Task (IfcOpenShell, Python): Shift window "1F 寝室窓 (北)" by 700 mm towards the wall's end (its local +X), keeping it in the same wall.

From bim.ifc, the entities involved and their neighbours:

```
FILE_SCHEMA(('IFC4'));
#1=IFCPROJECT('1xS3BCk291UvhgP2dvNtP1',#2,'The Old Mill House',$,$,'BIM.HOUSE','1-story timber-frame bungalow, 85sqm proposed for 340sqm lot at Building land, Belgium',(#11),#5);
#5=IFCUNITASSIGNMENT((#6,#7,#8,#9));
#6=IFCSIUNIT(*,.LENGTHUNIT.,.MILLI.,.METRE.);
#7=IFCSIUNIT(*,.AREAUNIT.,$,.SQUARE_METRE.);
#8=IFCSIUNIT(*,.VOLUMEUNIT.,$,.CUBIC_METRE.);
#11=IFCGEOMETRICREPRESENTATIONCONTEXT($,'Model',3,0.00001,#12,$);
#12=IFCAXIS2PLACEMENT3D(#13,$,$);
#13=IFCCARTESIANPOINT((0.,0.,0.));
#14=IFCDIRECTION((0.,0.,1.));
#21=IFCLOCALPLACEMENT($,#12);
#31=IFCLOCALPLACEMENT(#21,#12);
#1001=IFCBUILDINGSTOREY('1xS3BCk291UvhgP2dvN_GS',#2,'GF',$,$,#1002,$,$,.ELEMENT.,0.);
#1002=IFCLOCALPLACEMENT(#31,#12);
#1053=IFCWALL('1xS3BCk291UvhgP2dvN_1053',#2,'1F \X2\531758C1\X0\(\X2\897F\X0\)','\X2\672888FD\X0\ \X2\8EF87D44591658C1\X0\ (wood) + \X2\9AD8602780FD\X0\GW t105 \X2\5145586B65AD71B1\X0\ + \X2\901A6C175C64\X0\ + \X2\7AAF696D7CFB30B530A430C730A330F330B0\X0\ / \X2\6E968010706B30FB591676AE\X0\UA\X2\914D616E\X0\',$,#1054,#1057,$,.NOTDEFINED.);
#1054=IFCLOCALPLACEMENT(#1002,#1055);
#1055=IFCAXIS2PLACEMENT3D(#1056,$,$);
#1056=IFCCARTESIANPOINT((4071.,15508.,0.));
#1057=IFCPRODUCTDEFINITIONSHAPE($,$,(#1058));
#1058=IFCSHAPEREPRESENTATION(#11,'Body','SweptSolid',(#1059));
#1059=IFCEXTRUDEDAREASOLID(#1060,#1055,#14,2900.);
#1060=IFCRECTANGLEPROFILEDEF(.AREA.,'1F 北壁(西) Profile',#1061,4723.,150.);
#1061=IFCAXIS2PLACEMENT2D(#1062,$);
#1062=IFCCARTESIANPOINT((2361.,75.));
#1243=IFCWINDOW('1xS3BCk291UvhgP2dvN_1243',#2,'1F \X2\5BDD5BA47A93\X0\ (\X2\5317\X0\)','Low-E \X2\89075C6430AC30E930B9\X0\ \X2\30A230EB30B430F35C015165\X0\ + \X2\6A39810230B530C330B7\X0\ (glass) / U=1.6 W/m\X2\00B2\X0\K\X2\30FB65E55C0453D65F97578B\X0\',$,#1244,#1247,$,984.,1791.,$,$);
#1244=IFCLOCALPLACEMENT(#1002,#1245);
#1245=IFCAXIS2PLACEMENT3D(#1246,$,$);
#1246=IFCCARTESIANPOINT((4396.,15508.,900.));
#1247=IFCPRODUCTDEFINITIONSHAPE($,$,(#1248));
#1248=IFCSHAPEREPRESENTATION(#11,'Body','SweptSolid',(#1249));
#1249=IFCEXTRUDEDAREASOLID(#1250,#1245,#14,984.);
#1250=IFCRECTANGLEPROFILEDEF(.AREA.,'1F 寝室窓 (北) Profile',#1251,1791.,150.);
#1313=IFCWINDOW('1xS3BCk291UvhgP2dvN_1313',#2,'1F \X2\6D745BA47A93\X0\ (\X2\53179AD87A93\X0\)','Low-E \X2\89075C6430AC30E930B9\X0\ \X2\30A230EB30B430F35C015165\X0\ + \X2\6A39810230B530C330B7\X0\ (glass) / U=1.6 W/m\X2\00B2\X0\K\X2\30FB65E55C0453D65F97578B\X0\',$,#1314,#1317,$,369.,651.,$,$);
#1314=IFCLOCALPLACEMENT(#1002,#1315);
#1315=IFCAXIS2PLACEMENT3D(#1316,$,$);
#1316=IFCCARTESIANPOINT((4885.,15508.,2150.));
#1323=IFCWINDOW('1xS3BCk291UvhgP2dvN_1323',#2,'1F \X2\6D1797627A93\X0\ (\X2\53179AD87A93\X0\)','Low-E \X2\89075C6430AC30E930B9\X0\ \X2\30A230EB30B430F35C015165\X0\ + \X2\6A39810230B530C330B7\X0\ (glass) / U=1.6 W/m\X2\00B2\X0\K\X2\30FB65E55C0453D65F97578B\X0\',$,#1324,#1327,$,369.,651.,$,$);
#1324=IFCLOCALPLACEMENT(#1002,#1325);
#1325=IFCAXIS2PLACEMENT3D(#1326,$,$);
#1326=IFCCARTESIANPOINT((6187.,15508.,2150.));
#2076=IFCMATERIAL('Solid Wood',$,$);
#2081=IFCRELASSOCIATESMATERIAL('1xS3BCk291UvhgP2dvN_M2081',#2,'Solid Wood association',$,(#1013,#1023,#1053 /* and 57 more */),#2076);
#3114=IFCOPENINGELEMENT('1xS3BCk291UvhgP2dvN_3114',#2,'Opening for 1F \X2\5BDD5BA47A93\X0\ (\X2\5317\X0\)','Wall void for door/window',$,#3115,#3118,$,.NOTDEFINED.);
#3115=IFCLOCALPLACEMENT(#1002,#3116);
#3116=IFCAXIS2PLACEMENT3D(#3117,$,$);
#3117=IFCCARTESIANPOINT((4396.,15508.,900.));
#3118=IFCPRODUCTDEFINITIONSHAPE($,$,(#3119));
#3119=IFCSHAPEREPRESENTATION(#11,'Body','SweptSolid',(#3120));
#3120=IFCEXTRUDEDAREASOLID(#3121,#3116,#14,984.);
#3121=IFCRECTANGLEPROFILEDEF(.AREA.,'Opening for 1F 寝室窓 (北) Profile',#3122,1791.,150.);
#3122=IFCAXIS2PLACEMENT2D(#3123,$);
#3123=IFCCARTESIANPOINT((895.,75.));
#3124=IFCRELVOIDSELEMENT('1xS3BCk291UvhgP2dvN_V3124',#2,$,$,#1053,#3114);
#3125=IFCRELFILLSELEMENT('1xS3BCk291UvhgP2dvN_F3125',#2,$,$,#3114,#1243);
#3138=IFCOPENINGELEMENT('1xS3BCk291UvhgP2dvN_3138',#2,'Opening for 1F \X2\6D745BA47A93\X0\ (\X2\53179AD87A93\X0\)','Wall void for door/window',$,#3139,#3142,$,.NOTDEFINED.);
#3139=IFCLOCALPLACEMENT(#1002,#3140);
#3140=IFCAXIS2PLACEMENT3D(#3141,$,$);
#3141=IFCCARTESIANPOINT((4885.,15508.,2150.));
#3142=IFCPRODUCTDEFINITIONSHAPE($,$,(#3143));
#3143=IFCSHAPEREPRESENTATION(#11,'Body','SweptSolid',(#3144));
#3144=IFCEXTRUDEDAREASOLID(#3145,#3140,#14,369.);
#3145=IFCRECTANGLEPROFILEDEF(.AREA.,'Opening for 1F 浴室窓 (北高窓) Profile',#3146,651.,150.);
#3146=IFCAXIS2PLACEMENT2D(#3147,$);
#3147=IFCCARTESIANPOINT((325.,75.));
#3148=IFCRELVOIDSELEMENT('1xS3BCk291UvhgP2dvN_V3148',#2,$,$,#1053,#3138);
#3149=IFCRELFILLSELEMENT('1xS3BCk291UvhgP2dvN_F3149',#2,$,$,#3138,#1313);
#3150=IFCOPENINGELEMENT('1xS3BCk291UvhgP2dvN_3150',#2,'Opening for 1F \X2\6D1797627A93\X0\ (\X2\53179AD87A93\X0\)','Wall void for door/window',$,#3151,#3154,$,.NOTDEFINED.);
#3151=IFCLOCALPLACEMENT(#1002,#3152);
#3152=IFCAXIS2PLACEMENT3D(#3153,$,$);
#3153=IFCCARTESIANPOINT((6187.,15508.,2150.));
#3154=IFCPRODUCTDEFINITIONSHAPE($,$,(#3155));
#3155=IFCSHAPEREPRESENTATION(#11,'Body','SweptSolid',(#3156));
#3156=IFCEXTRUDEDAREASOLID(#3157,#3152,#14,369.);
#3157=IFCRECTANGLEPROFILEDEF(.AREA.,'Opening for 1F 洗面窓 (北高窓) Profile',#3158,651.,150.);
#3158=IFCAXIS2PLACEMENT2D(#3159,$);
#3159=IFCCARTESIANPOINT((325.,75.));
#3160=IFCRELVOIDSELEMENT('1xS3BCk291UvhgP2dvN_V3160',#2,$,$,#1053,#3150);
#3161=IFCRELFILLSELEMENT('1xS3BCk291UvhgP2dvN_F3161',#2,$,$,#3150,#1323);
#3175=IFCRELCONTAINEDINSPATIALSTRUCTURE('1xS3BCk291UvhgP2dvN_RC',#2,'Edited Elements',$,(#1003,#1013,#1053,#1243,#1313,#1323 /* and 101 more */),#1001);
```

```python
import ifcopenshell
import ifcopenshell.api.geometry
import ifcopenshell.util.placement
import ifcopenshell.util.unit

model = ifcopenshell.open("bim.ifc")
unit_scale = ifcopenshell.util.unit.calculate_unit_scale(model)

window = model.by_guid("1xS3BCk291UvhgP2dvN_1243")
opening = window.FillsVoids[0].RelatingOpeningElement
wall = opening.VoidsElements[0].RelatingBuildingElement

wall_matrix = ifcopenshell.util.placement.get_local_placement(wall.ObjectPlacement)
shift = wall_matrix[:3, 0] * 0.7 / unit_scale
before = ifcopenshell.util.placement.get_local_placement(window.ObjectPlacement)[:3, 3].copy()

# The window is not placed relative to its opening, so move both.
for product in (opening, window):
    matrix = ifcopenshell.util.placement.get_local_placement(product.ObjectPlacement)
    matrix[:3, 3] += shift
    ifcopenshell.api.geometry.edit_object_placement(model, product=product, matrix=matrix, is_si=False)

after = ifcopenshell.util.placement.get_local_placement(window.ObjectPlacement)[:3, 3]
print("window moved by", (after - before).round(3) + 0.0)

model.write("bim_v2.ifc")
```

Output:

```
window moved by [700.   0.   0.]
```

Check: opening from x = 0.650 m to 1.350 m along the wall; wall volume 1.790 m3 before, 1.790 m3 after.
